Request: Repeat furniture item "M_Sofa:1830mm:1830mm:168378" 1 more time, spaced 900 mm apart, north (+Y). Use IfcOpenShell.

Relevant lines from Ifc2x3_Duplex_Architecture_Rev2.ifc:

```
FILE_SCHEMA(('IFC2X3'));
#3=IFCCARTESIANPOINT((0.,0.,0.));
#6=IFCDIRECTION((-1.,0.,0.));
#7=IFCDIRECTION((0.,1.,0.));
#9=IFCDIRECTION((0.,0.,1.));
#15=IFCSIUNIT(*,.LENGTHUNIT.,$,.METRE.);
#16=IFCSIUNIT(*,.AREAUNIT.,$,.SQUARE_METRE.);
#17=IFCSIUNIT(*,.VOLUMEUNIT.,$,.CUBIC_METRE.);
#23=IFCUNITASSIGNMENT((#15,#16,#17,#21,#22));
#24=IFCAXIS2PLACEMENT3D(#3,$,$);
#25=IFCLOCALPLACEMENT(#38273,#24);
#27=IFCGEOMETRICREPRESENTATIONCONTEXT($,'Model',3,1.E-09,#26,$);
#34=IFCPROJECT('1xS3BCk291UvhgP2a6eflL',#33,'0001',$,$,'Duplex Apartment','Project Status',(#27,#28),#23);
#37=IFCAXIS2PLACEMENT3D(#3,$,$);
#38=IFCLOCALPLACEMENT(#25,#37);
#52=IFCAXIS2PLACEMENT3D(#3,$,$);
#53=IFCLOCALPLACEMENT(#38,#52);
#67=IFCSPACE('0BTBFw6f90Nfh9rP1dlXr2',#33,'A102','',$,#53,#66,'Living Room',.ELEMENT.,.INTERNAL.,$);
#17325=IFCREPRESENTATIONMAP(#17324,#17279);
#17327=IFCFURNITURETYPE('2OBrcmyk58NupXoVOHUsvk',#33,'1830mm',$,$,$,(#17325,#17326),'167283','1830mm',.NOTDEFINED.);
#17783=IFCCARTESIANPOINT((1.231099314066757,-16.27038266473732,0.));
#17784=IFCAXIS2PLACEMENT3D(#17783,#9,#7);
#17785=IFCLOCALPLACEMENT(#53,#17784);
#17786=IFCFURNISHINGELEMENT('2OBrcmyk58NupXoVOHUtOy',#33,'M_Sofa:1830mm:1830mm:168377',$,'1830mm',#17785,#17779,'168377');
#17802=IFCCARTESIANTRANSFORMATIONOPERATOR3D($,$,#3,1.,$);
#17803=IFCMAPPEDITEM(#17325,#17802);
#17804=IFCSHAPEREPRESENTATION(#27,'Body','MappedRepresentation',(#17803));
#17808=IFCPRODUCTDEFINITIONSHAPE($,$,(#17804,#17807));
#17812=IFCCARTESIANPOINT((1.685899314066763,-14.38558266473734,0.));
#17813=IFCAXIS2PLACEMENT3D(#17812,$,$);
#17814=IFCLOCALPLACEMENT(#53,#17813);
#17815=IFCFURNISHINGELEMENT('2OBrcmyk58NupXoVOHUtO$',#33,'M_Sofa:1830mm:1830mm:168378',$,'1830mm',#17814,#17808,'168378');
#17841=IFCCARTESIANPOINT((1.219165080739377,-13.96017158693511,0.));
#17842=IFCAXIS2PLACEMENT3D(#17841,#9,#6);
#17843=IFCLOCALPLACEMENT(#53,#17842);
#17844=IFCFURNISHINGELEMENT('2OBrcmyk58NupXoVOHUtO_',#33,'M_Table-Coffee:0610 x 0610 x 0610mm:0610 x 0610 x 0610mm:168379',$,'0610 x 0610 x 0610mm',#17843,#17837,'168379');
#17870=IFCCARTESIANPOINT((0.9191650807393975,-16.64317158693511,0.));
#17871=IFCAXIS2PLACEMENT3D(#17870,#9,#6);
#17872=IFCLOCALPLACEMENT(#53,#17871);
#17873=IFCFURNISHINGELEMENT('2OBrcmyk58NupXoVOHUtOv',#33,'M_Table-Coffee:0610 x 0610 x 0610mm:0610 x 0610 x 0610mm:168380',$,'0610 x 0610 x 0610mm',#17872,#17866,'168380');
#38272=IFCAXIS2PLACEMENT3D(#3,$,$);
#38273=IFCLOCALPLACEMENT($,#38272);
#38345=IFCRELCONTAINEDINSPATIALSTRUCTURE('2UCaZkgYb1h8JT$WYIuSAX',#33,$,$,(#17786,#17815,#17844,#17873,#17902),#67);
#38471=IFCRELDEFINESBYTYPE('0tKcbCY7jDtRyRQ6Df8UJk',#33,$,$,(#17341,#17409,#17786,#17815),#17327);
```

```python
import numpy as np
import ifcopenshell
import ifcopenshell.api.geometry
import ifcopenshell.api.root
import ifcopenshell.util.element
import ifcopenshell.util.placement
import ifcopenshell.util.unit

model = ifcopenshell.open("Ifc2x3_Duplex_Architecture_Rev2.ifc")
unit_scale = ifcopenshell.util.unit.calculate_unit_scale(model)


def reuse_history(source, copy):
    """copy_class also copies each property set's owner history, people and application; keep the originals."""
    for rel in copy.IsDefinedBy:
        if rel.is_a("IfcRelDefinesByProperties") and (history := rel.RelatingPropertyDefinition.OwnerHistory):
            rel.RelatingPropertyDefinition.OwnerHistory = source.OwnerHistory
            ifcopenshell.util.element.remove_deep2(model, history)


source = model.by_guid("2OBrcmyk58NupXoVOHUtO$")
base = ifcopenshell.util.placement.get_local_placement(source.ObjectPlacement)
step = np.array([0.0, 1.0, 0.0]) * 0.9 / unit_scale

for i in range(1, 2):
    copy = ifcopenshell.api.root.copy_class(model, product=source)
    copy.Representation = ifcopenshell.util.element.copy_deep(
        model, source.Representation, exclude=["IfcGeometricRepresentationContext", "IfcRepresentationMap"]
    )
    copy.Name = "M_Sofa:1830mm:1830mm"
    copy.Tag = None
    reuse_history(source, copy)
    matrix = base.copy()
    matrix[:3, 3] += i * step
    print("added at", matrix[:3, 3].round(3) + 0.0)
    ifcopenshell.api.geometry.edit_object_placement(model, product=copy, matrix=matrix, is_si=False)

model.write("Ifc2x3_Duplex_Architecture_Rev2-out.ifc")
```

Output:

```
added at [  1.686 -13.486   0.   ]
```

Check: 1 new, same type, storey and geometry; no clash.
